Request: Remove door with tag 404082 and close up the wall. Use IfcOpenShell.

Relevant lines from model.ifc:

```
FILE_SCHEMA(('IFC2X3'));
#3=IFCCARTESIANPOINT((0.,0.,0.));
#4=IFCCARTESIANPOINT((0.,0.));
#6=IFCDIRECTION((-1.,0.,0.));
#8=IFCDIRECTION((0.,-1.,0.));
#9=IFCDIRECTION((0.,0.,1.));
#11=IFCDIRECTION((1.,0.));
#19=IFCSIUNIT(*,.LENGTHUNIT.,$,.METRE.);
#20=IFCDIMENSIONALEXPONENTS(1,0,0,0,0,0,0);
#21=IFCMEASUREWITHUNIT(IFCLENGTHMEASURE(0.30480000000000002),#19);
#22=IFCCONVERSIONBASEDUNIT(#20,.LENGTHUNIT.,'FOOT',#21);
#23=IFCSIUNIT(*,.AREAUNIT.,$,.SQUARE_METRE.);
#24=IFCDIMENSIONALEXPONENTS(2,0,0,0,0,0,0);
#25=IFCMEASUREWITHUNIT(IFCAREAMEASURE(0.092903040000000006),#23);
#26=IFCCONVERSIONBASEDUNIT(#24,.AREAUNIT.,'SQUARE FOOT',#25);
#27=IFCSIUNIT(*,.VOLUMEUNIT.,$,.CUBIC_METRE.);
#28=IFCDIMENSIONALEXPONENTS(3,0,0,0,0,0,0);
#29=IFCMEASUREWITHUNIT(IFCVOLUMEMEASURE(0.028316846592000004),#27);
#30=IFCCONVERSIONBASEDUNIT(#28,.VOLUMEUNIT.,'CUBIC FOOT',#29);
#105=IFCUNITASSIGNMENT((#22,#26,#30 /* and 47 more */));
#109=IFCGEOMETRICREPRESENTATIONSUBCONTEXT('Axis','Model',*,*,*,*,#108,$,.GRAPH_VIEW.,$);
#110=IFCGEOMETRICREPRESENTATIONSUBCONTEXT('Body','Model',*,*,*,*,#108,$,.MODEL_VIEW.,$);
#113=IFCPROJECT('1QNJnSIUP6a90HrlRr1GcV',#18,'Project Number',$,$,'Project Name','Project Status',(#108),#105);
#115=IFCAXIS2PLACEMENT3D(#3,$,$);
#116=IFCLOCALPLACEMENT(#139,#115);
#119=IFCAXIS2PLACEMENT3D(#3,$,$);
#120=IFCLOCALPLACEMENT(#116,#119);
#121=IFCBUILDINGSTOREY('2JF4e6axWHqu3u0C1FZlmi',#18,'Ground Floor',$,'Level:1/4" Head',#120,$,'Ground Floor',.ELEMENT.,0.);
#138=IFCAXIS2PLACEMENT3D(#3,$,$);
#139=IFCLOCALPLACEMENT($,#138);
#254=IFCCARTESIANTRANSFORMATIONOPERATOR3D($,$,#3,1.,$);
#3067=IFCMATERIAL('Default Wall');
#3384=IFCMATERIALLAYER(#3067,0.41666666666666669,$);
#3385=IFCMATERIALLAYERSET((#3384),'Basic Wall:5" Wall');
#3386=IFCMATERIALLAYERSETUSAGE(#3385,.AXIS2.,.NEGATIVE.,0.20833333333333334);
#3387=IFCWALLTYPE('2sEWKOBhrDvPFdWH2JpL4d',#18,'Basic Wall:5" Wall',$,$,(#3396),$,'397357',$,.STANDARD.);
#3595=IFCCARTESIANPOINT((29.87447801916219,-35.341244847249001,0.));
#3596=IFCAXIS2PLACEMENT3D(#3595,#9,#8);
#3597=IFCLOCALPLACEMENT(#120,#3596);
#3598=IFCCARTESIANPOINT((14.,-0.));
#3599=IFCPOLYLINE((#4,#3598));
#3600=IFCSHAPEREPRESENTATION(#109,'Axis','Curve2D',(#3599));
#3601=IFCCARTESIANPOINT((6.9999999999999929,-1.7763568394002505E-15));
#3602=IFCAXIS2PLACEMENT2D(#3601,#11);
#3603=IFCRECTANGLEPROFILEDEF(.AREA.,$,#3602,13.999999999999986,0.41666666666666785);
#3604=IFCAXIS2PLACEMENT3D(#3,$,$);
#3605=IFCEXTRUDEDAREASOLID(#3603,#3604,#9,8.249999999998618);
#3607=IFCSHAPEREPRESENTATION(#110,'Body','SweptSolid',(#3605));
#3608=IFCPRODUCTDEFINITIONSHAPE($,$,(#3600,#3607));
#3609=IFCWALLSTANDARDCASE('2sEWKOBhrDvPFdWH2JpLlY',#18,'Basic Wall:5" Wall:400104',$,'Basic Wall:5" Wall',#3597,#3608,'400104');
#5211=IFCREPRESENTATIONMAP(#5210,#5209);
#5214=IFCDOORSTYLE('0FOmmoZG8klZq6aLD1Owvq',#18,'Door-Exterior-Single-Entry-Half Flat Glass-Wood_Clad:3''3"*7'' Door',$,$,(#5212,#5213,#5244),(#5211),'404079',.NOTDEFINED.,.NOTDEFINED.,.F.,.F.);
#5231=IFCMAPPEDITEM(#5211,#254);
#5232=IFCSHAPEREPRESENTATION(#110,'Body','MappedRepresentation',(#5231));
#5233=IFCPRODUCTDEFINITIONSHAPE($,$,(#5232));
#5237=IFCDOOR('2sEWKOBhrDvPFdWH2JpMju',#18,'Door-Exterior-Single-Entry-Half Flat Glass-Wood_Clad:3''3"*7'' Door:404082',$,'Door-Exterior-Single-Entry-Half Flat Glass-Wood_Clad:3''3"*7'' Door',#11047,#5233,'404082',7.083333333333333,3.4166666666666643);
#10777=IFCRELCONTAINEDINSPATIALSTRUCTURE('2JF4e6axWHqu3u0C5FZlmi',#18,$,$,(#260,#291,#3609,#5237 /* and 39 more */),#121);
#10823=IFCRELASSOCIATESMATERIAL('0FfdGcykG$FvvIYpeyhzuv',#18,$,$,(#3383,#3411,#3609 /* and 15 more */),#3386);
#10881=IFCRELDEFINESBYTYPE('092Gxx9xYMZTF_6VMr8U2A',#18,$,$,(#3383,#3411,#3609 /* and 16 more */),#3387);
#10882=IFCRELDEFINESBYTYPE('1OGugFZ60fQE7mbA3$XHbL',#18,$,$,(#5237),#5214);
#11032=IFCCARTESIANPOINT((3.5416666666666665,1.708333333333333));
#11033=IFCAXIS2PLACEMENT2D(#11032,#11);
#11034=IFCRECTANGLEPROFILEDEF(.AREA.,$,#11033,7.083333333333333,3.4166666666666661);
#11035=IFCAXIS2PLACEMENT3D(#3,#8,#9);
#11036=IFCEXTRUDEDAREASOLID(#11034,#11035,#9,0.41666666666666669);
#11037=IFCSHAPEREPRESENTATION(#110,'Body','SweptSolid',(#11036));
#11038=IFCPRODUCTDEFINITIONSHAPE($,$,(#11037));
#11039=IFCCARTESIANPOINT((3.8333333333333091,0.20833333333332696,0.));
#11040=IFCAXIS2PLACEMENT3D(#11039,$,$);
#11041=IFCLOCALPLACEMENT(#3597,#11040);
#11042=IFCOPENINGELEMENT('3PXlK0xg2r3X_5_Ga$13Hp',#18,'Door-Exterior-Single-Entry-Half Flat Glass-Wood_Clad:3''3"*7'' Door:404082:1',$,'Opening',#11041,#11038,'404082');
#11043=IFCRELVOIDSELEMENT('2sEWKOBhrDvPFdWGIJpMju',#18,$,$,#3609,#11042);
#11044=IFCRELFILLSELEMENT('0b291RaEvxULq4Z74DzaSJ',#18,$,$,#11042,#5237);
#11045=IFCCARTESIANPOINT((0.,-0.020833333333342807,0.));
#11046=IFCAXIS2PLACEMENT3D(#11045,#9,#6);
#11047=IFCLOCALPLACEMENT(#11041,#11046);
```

```python
import ifcopenshell
import ifcopenshell.api.feature
import ifcopenshell.api.root
import ifcopenshell.geom
import ifcopenshell.util.shape

model = ifcopenshell.open("model.ifc")
settings = ifcopenshell.geom.settings()


def volume(element):
    """Net volume in cubic metres, openings subtracted."""
    shape = ifcopenshell.geom.create_shape(settings, element)
    return ifcopenshell.util.shape.get_volume(shape.geometry)


door = model.by_id(5237)
opening = door.FillsVoids[0].RelatingOpeningElement
wall = opening.VoidsElements[0].RelatingBuildingElement
before = volume(wall)

ifcopenshell.api.root.remove_product(model, product=door)
ifcopenshell.api.feature.remove_feature(model, feature=opening)

after = volume(wall)

print(f"wall volume {before:.3f} -> {after:.3f} m3")

model.write("model-out.ifc")
```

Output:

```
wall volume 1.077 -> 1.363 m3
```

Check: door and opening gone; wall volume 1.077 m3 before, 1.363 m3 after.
